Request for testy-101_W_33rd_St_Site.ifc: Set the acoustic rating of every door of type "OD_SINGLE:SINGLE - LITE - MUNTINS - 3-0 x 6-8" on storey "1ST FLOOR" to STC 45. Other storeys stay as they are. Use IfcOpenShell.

First a look at what the model holds.

```python
import ifcopenshell
import ifcopenshell.util.element

model = ifcopenshell.open("testy-101_W_33rd_St_Site.ifc")
print(model.schema)
storey = next(s for s in model.by_type("IfcBuildingStorey") if s.Name == "1ST FLOOR")
doors = [e for e in ifcopenshell.util.element.get_decomposition(storey) if e.is_a("IfcDoor")]
seen = {}
for e in doors:
    element_type = ifcopenshell.util.element.get_type(e)
    key = (element_type.Name if element_type != e and element_type else None, ifcopenshell.util.element.get_pset(e, "Pset_DoorCommon", "AcousticRating"))
    seen[key] = seen.get(key, 0) + 1
for (name, value), count in sorted(seen.items(), key=str):
    print(count, "x", name, "|", value)
```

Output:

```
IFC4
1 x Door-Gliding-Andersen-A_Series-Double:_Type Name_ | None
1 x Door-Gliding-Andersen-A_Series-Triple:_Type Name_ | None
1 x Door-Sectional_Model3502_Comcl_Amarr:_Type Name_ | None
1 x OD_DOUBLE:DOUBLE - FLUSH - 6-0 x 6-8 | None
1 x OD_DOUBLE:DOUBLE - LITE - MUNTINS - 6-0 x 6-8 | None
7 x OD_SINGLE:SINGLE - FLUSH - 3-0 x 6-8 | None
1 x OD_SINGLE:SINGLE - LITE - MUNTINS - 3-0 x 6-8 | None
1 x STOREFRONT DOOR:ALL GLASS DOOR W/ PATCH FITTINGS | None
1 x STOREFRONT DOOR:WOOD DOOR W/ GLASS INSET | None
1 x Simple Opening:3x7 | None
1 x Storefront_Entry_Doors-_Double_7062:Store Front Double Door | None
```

```python
import ifcopenshell
import ifcopenshell.api.pset
import ifcopenshell.util.element

model = ifcopenshell.open("testy-101_W_33rd_St_Site.ifc")

storey = next(s for s in model.by_type("IfcBuildingStorey") if s.Name == "1ST FLOOR")
doors = [e for e in ifcopenshell.util.element.get_decomposition(storey) if e.is_a("IfcDoor")]

count = 0
for e in doors:
    element_type = ifcopenshell.util.element.get_type(e)
    if element_type in (None, e) or element_type.Name != "OD_SINGLE:SINGLE - LITE - MUNTINS - 3-0 x 6-8":
        continue
    # add_pset returns the element's existing set when there is one.
    pset = ifcopenshell.api.pset.add_pset(model, product=e, name="Pset_DoorCommon")
    ifcopenshell.api.pset.edit_pset(model, pset=pset, properties={"AcousticRating": "STC 45"})
    count += 1

print(count, "doors updated")

model.write("testy-101_W_33rd_St_Site_v2.ifc")
```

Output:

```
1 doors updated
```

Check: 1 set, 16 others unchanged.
